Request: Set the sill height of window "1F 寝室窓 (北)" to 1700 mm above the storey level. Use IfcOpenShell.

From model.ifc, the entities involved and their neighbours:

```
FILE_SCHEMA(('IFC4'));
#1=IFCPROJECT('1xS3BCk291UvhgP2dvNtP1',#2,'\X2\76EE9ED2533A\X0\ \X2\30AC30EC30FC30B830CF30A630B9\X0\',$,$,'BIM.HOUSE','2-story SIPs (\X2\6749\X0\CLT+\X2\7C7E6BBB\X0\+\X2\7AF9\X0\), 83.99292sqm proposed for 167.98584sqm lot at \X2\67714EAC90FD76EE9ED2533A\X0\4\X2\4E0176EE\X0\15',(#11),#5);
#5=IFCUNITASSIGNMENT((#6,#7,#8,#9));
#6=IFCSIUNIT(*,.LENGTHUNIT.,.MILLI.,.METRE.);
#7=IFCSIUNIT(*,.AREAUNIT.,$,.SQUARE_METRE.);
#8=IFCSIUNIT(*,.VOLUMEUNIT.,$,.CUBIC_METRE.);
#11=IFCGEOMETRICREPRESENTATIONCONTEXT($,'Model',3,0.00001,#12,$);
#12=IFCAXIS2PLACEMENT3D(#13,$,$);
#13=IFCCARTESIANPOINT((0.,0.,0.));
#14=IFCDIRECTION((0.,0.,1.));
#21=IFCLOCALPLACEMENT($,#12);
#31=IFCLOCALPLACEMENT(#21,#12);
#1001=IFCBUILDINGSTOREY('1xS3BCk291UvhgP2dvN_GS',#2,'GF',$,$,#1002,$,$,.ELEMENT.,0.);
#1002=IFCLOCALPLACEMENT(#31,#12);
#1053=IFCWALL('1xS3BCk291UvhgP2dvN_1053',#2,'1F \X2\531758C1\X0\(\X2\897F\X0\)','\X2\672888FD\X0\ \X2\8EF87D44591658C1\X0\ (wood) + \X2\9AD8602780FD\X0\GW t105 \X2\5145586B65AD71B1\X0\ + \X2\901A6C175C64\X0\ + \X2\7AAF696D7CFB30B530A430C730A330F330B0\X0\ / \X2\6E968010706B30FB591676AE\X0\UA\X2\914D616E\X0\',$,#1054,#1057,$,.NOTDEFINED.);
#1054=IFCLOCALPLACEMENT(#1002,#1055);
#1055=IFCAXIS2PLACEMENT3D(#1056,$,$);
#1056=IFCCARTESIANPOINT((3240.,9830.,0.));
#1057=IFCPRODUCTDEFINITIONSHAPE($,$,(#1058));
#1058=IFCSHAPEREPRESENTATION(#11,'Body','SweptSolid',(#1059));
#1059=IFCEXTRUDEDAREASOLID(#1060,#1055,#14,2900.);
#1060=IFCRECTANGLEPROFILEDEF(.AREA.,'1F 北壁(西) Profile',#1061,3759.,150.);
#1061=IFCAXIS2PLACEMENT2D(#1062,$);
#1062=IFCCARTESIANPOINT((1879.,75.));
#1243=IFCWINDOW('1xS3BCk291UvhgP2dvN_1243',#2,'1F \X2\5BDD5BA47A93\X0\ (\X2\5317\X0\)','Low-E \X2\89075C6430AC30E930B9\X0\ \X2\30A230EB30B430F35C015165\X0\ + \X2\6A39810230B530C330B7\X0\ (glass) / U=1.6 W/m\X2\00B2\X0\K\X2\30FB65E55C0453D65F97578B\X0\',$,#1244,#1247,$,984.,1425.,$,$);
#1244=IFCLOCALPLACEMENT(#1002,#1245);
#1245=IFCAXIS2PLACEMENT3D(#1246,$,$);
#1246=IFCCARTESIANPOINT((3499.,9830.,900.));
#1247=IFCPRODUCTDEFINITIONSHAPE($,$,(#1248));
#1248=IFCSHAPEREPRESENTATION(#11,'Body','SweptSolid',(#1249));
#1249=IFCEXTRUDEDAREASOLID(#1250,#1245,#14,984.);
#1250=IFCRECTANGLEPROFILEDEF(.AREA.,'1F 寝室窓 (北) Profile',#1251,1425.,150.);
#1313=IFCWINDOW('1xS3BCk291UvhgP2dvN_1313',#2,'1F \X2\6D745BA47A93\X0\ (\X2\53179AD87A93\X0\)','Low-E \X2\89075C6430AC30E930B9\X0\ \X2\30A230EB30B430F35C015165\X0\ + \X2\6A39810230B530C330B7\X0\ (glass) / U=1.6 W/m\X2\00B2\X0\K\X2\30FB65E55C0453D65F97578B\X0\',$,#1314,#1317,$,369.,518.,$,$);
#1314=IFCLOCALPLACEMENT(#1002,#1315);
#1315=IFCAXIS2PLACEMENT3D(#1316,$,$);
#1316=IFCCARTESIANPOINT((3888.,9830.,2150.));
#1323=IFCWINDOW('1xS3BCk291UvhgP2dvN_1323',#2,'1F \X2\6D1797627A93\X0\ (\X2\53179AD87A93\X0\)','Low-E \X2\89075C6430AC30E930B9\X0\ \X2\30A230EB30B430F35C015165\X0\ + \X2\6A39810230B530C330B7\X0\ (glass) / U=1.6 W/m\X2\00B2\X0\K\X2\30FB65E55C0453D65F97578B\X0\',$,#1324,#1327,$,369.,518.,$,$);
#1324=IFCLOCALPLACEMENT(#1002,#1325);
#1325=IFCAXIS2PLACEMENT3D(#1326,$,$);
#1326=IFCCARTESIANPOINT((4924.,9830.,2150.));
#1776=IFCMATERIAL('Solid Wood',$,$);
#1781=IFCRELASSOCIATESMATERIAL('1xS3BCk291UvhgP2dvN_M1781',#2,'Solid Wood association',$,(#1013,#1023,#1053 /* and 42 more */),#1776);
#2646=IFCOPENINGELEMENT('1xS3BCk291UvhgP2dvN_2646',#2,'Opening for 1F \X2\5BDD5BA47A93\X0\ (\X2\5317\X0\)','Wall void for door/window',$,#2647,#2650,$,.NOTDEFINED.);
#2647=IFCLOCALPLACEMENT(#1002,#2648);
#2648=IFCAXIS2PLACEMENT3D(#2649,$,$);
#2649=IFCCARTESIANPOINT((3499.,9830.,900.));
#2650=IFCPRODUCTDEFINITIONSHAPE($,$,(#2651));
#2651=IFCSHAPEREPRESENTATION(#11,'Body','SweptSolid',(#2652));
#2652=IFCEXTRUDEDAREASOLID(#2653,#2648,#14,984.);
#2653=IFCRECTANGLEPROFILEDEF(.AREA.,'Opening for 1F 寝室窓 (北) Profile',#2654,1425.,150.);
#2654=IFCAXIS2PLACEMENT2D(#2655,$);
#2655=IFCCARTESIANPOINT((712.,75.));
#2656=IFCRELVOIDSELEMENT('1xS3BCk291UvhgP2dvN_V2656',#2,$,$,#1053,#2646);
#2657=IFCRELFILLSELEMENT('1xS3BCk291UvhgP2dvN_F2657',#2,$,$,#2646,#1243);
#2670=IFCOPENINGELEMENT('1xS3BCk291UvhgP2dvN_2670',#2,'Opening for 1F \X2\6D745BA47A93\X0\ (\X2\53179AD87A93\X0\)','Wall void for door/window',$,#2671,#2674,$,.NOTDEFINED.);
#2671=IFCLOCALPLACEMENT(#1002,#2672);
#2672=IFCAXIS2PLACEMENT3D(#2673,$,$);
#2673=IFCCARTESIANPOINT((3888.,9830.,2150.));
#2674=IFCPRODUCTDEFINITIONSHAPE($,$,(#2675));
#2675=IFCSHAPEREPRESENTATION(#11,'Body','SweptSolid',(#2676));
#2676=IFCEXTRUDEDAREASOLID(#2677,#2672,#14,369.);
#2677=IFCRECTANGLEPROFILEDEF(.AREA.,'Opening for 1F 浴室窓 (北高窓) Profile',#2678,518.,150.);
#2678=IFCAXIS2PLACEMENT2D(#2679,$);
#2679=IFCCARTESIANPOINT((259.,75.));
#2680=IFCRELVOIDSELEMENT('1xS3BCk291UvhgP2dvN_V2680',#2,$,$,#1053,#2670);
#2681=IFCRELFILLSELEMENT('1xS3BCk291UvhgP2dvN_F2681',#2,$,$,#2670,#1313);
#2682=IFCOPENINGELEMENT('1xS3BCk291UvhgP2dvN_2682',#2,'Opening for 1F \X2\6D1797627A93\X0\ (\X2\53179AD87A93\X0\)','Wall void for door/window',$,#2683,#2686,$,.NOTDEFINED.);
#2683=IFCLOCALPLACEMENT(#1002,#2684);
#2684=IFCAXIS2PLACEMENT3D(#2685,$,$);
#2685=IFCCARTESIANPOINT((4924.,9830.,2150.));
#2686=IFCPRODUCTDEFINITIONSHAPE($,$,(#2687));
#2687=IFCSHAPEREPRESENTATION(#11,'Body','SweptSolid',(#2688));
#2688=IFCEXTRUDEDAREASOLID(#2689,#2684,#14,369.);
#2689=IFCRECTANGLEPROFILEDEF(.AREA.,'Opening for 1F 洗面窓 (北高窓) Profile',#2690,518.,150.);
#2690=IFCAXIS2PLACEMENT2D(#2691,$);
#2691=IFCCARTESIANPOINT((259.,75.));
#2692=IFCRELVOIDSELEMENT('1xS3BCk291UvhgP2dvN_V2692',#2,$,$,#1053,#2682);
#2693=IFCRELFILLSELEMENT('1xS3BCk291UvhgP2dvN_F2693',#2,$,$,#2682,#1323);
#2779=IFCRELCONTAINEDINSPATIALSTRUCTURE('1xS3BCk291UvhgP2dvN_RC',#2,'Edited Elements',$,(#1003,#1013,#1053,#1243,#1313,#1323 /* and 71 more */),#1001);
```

```python
import numpy as np
import ifcopenshell
import ifcopenshell.api.geometry
import ifcopenshell.geom
import ifcopenshell.util.element
import ifcopenshell.util.placement
import ifcopenshell.util.shape
import ifcopenshell.util.unit

model = ifcopenshell.open("model.ifc")
unit_scale = ifcopenshell.util.unit.calculate_unit_scale(model)

window = model.by_guid("1xS3BCk291UvhgP2dvN_1243")
opening = window.FillsVoids[0].RelatingOpeningElement
storey = ifcopenshell.util.element.get_container(window, ifc_class="IfcBuildingStorey")
level = ifcopenshell.util.placement.get_local_placement(storey.ObjectPlacement)[2, 3]

# The opening's origin need not be at the sill, so measure its lowest point.
shape = ifcopenshell.geom.create_shape(ifcopenshell.geom.settings(), opening)
bottom = ifcopenshell.util.shape.get_shape_bottom_elevation(shape, shape.geometry) / unit_scale
dz = level + 1.7 / unit_scale - bottom

shift = np.array([0.0, 0.0, dz])
# The window is not placed relative to its opening, so move both.
for product in (opening, window):
    matrix = ifcopenshell.util.placement.get_local_placement(product.ObjectPlacement)
    matrix[:3, 3] += shift
    ifcopenshell.api.geometry.edit_object_placement(model, product=product, matrix=matrix, is_si=False)

print(f"moved by {dz * unit_scale:+.3f} m")

model.write("model-out.ifc")
```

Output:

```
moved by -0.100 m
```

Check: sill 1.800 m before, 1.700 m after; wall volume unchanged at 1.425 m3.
